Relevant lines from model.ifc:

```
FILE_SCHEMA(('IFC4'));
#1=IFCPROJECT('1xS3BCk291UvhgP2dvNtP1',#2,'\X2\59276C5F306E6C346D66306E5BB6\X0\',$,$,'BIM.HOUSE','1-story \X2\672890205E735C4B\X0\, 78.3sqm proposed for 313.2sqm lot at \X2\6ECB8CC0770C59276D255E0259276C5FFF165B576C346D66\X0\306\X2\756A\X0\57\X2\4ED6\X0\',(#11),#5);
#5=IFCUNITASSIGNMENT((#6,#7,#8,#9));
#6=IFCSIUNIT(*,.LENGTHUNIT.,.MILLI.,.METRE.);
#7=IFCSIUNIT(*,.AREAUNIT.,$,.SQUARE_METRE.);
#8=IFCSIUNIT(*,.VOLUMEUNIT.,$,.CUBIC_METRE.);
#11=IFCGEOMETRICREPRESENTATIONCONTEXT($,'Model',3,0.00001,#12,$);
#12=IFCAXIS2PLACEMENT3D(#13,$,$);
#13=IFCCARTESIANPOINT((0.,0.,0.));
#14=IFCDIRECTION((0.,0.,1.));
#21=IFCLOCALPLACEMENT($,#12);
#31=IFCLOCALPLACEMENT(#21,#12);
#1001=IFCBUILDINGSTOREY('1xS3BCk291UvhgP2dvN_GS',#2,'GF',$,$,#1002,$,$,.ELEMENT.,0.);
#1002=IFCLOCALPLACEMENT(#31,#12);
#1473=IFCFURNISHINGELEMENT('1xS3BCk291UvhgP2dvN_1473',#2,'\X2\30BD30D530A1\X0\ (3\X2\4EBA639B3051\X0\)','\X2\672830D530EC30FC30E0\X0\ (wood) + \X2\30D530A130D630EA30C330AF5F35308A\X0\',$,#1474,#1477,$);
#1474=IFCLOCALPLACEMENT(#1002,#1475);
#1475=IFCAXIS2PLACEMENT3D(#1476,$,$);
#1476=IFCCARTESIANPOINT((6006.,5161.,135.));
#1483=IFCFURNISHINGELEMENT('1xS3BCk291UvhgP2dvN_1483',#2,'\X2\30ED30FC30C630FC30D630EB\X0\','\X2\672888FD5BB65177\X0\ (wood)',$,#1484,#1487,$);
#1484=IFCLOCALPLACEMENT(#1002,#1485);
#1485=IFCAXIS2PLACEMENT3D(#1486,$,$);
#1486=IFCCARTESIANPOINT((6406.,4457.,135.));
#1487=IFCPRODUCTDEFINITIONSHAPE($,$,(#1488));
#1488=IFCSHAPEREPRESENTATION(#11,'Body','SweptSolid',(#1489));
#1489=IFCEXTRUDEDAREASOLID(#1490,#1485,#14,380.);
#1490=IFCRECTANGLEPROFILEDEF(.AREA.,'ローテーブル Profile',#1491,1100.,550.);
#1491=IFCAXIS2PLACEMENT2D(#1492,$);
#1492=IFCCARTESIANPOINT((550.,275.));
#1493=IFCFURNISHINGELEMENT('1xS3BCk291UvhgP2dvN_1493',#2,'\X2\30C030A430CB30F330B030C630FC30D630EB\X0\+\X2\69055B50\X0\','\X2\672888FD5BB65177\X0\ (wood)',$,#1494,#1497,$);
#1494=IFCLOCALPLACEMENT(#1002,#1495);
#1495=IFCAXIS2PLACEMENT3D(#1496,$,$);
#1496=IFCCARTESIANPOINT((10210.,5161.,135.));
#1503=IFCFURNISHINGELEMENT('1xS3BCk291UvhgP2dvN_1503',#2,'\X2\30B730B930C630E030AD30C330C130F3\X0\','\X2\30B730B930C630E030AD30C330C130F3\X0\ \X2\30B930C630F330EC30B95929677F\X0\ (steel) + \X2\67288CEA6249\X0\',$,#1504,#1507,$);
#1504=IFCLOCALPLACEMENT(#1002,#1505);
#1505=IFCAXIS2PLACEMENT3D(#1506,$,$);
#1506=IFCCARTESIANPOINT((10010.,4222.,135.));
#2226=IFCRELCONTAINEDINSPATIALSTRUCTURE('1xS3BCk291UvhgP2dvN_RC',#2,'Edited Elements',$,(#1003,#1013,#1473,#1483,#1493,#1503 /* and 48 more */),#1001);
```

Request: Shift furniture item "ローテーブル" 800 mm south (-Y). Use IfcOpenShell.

```python
import ifcopenshell
import ifcopenshell.api.geometry
import ifcopenshell.util.placement
import ifcopenshell.util.unit

model = ifcopenshell.open("model.ifc")
unit_scale = ifcopenshell.util.unit.calculate_unit_scale(model)

item = model.by_guid("1xS3BCk291UvhgP2dvN_1483")
matrix = ifcopenshell.util.placement.get_local_placement(item.ObjectPlacement)
matrix[1, 3] -= 0.8 / unit_scale
ifcopenshell.api.geometry.edit_object_placement(model, product=item, matrix=matrix, is_si=False)

print(ifcopenshell.util.placement.get_local_placement(item.ObjectPlacement).round(3) + 0.0)

model.write("model_edited.ifc")
```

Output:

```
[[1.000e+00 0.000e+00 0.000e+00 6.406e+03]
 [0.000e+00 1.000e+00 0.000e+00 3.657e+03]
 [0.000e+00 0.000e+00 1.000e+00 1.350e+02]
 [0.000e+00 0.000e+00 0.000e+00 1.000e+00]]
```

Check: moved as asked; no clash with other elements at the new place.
